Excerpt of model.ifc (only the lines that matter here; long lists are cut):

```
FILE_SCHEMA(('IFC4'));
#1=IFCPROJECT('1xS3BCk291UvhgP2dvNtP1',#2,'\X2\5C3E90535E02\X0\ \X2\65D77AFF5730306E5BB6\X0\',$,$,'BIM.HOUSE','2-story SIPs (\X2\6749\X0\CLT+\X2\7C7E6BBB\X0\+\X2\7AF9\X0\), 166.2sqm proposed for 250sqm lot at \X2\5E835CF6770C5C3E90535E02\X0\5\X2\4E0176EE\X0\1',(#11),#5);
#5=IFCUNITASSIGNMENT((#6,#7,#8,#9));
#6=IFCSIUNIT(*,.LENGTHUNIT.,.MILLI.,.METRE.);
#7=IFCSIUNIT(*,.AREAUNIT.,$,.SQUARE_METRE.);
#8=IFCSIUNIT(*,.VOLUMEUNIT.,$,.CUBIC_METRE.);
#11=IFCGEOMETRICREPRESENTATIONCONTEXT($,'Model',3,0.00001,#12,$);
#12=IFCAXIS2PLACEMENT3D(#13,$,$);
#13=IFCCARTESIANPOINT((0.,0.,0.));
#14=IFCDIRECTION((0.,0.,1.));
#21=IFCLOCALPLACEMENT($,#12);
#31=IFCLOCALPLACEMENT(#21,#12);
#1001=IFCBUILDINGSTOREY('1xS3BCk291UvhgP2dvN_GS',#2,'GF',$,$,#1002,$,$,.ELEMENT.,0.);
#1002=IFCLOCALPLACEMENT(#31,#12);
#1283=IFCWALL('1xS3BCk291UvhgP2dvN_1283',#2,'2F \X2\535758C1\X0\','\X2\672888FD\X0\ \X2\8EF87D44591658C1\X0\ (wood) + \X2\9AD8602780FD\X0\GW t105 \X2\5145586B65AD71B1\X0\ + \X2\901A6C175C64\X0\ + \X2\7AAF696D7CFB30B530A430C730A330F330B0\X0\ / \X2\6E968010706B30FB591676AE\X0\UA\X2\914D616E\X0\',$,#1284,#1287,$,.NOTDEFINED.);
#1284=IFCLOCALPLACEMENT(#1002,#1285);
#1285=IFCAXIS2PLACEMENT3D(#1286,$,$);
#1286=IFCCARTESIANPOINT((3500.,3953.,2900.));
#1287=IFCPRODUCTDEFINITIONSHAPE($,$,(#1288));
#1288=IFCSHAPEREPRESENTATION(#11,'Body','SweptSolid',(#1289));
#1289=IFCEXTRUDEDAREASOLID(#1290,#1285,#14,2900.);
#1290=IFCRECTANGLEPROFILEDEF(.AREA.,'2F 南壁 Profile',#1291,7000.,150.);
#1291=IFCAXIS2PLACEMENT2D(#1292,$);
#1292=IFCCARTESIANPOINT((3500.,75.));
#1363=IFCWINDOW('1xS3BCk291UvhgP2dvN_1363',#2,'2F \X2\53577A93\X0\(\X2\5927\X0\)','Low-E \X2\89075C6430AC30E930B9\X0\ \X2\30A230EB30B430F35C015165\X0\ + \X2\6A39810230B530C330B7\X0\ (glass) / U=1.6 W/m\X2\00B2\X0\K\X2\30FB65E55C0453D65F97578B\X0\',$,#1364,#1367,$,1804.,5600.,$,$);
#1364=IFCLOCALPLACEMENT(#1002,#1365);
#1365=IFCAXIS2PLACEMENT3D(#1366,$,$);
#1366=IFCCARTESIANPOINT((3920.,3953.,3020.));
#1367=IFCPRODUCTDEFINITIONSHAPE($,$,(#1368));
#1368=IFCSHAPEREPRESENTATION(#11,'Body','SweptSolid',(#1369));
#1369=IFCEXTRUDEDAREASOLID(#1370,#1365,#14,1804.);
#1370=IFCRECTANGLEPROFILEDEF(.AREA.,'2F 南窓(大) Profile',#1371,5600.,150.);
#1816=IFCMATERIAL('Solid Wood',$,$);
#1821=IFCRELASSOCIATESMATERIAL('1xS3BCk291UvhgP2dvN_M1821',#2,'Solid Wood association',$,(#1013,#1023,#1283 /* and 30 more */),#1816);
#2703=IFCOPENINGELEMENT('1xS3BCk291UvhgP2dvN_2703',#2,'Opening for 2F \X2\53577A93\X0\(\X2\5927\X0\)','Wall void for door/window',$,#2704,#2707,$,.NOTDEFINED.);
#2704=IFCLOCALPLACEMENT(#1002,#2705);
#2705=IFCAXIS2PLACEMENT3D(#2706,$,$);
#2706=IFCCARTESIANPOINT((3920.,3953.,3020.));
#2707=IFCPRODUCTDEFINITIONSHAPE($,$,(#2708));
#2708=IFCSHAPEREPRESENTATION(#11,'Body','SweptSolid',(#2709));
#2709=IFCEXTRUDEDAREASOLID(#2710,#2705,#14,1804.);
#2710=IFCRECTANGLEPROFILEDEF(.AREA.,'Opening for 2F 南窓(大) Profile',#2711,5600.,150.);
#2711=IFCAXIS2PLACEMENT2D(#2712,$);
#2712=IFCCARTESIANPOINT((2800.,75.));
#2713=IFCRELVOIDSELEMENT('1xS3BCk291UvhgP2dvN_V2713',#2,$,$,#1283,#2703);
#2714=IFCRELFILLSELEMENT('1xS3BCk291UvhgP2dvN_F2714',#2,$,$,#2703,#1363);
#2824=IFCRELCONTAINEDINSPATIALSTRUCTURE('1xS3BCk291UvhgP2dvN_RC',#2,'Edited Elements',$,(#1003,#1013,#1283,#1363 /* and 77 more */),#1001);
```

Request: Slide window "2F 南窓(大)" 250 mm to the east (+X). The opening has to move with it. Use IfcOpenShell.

```python
import ifcopenshell
import ifcopenshell.api.geometry
import ifcopenshell.util.placement
import ifcopenshell.util.unit

model = ifcopenshell.open("model.ifc")
unit_scale = ifcopenshell.util.unit.calculate_unit_scale(model)

window = model.by_guid("1xS3BCk291UvhgP2dvN_1363")
opening = window.FillsVoids[0].RelatingOpeningElement
wall = opening.VoidsElements[0].RelatingBuildingElement

wall_matrix = ifcopenshell.util.placement.get_local_placement(wall.ObjectPlacement)
shift = wall_matrix[:3, 0] * 0.25 / unit_scale
before = ifcopenshell.util.placement.get_local_placement(window.ObjectPlacement)[:3, 3].copy()

# The window is not placed relative to its opening, so move both.
for product in (opening, window):
    matrix = ifcopenshell.util.placement.get_local_placement(product.ObjectPlacement)
    matrix[:3, 3] += shift
    ifcopenshell.api.geometry.edit_object_placement(model, product=product, matrix=matrix, is_si=False)

after = ifcopenshell.util.placement.get_local_placement(window.ObjectPlacement)[:3, 3]
print("window moved by", (after - before).round(3) + 0.0)

model.write("model_rev.ifc")
```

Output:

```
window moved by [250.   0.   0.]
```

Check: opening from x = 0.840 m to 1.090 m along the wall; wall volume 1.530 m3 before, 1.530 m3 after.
